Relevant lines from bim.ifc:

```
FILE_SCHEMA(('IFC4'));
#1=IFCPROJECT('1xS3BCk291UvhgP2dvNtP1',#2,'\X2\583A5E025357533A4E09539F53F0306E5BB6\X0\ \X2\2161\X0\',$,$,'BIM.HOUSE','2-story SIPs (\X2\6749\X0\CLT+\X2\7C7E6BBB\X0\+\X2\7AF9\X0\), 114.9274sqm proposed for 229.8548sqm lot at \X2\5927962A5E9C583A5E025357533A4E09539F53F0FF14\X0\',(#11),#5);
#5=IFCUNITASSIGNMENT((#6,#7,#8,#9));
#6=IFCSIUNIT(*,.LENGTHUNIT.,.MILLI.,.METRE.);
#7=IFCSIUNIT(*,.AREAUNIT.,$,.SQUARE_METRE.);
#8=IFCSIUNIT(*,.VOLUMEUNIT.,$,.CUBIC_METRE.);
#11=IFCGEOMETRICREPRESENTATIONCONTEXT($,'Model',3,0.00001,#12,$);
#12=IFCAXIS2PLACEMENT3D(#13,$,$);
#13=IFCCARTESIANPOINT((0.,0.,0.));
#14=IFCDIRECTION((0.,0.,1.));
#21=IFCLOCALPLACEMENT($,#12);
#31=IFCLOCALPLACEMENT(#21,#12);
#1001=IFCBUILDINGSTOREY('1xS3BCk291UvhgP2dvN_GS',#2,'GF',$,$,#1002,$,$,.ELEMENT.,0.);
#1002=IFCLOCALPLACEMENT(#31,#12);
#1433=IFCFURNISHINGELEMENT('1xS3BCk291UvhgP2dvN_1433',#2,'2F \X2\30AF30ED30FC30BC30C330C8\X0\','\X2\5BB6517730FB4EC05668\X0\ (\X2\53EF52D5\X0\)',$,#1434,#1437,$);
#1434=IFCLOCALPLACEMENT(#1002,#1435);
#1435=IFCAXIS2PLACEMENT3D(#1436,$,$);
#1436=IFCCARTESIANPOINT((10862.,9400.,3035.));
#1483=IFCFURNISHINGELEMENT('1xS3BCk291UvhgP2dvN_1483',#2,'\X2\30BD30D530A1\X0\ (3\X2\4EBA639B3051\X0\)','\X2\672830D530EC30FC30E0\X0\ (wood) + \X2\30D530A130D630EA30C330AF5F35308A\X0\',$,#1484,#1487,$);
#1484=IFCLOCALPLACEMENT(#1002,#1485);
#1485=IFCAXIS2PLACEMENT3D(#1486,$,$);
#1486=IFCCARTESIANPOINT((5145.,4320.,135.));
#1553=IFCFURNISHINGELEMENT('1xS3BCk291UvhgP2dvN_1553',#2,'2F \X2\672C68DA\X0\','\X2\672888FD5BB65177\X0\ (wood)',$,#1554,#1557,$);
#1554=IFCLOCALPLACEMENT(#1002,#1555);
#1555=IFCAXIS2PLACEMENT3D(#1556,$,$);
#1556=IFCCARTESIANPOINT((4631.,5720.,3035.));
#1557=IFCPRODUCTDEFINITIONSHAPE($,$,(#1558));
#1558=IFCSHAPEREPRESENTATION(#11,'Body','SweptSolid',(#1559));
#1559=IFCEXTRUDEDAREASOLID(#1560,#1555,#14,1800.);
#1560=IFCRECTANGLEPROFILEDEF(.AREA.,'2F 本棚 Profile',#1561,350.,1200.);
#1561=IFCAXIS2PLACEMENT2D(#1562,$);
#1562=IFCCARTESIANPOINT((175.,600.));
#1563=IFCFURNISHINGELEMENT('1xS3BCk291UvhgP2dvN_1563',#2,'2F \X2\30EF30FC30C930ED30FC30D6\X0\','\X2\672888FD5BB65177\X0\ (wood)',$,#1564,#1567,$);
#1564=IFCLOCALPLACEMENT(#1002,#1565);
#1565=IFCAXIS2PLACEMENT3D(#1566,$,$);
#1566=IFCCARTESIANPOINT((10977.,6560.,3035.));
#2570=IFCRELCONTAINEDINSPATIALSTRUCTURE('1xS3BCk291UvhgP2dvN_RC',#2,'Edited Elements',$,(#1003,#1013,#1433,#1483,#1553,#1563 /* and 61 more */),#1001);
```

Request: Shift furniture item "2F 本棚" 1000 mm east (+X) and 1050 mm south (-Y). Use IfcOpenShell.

```python
import ifcopenshell
import ifcopenshell.api.geometry
import ifcopenshell.util.placement

model = ifcopenshell.open("bim.ifc")

item = model.by_guid("1xS3BCk291UvhgP2dvN_1553")
matrix = ifcopenshell.util.placement.get_local_placement(item.ObjectPlacement)
matrix[0, 3] += 1000.0
matrix[1, 3] -= 1050.0
ifcopenshell.api.geometry.edit_object_placement(model, product=item, matrix=matrix, is_si=False)

print(ifcopenshell.util.placement.get_local_placement(item.ObjectPlacement).round(3) + 0.0)

model.write("bim_v2.ifc")
```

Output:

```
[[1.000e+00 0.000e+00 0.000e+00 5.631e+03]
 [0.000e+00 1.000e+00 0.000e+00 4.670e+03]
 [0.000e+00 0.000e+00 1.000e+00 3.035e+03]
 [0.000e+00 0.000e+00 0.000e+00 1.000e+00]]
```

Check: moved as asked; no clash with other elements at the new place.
